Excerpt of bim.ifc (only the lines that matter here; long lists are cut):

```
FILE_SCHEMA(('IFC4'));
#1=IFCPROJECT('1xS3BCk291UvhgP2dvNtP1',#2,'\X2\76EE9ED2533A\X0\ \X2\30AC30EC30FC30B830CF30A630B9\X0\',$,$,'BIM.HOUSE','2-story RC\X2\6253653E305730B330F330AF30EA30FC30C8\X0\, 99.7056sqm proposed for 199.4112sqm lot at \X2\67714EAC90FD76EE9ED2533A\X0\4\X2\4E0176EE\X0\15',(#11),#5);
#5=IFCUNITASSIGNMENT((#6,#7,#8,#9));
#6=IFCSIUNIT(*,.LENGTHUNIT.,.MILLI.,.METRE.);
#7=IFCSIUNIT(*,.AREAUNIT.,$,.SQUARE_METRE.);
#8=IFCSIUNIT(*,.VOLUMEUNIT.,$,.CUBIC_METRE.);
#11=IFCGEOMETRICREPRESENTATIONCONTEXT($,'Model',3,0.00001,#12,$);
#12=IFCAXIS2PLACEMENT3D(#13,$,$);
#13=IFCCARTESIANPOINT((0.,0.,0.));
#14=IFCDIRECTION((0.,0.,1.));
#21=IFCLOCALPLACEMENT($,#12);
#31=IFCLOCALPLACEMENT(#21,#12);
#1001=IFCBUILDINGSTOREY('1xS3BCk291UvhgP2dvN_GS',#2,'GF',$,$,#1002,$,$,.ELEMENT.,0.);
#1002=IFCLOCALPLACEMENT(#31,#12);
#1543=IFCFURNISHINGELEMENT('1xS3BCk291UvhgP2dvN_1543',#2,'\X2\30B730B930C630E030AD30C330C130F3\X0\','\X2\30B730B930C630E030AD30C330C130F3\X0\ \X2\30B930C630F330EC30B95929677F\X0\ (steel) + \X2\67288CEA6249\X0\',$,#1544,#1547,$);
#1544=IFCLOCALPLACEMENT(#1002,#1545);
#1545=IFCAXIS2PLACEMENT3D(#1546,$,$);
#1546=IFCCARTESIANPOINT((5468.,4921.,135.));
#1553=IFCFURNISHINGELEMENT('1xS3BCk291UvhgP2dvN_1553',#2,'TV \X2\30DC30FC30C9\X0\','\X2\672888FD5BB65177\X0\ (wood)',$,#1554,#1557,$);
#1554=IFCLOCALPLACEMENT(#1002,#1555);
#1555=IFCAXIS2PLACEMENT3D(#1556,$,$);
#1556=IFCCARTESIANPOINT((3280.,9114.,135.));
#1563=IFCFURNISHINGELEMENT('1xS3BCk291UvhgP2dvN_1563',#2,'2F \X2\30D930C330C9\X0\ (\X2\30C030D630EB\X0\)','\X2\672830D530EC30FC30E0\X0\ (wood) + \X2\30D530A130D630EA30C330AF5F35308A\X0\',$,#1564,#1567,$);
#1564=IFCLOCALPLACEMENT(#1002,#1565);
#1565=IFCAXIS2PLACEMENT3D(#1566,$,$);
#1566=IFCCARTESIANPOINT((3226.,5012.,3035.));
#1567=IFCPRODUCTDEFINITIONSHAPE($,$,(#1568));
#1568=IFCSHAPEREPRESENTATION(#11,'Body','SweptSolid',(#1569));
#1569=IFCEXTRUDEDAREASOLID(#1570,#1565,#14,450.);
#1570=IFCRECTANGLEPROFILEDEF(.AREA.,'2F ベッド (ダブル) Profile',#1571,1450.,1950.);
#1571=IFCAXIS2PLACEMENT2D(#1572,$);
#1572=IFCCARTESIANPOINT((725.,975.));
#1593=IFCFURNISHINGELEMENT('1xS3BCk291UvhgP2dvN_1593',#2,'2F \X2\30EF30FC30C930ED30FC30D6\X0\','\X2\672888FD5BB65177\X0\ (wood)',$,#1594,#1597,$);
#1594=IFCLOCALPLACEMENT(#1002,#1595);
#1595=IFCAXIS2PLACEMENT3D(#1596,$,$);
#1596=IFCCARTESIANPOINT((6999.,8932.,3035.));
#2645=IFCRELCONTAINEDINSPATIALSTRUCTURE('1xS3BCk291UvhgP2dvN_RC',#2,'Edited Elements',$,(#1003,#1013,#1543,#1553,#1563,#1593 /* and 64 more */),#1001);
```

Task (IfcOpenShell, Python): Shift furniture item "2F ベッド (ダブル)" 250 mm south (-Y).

```python
import ifcopenshell
import ifcopenshell.api.geometry
import ifcopenshell.util.placement
import ifcopenshell.util.unit

model = ifcopenshell.open("bim.ifc")
unit_scale = ifcopenshell.util.unit.calculate_unit_scale(model)

item = model.by_guid("1xS3BCk291UvhgP2dvN_1563")
matrix = ifcopenshell.util.placement.get_local_placement(item.ObjectPlacement)
matrix[1, 3] -= 0.25 / unit_scale
ifcopenshell.api.geometry.edit_object_placement(model, product=item, matrix=matrix, is_si=False)

print(ifcopenshell.util.placement.get_local_placement(item.ObjectPlacement).round(3) + 0.0)

model.write("bim_v2.ifc")
```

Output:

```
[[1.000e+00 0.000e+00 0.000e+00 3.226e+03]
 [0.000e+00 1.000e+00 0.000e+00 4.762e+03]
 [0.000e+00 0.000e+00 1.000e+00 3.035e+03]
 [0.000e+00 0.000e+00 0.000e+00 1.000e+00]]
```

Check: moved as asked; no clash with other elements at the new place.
